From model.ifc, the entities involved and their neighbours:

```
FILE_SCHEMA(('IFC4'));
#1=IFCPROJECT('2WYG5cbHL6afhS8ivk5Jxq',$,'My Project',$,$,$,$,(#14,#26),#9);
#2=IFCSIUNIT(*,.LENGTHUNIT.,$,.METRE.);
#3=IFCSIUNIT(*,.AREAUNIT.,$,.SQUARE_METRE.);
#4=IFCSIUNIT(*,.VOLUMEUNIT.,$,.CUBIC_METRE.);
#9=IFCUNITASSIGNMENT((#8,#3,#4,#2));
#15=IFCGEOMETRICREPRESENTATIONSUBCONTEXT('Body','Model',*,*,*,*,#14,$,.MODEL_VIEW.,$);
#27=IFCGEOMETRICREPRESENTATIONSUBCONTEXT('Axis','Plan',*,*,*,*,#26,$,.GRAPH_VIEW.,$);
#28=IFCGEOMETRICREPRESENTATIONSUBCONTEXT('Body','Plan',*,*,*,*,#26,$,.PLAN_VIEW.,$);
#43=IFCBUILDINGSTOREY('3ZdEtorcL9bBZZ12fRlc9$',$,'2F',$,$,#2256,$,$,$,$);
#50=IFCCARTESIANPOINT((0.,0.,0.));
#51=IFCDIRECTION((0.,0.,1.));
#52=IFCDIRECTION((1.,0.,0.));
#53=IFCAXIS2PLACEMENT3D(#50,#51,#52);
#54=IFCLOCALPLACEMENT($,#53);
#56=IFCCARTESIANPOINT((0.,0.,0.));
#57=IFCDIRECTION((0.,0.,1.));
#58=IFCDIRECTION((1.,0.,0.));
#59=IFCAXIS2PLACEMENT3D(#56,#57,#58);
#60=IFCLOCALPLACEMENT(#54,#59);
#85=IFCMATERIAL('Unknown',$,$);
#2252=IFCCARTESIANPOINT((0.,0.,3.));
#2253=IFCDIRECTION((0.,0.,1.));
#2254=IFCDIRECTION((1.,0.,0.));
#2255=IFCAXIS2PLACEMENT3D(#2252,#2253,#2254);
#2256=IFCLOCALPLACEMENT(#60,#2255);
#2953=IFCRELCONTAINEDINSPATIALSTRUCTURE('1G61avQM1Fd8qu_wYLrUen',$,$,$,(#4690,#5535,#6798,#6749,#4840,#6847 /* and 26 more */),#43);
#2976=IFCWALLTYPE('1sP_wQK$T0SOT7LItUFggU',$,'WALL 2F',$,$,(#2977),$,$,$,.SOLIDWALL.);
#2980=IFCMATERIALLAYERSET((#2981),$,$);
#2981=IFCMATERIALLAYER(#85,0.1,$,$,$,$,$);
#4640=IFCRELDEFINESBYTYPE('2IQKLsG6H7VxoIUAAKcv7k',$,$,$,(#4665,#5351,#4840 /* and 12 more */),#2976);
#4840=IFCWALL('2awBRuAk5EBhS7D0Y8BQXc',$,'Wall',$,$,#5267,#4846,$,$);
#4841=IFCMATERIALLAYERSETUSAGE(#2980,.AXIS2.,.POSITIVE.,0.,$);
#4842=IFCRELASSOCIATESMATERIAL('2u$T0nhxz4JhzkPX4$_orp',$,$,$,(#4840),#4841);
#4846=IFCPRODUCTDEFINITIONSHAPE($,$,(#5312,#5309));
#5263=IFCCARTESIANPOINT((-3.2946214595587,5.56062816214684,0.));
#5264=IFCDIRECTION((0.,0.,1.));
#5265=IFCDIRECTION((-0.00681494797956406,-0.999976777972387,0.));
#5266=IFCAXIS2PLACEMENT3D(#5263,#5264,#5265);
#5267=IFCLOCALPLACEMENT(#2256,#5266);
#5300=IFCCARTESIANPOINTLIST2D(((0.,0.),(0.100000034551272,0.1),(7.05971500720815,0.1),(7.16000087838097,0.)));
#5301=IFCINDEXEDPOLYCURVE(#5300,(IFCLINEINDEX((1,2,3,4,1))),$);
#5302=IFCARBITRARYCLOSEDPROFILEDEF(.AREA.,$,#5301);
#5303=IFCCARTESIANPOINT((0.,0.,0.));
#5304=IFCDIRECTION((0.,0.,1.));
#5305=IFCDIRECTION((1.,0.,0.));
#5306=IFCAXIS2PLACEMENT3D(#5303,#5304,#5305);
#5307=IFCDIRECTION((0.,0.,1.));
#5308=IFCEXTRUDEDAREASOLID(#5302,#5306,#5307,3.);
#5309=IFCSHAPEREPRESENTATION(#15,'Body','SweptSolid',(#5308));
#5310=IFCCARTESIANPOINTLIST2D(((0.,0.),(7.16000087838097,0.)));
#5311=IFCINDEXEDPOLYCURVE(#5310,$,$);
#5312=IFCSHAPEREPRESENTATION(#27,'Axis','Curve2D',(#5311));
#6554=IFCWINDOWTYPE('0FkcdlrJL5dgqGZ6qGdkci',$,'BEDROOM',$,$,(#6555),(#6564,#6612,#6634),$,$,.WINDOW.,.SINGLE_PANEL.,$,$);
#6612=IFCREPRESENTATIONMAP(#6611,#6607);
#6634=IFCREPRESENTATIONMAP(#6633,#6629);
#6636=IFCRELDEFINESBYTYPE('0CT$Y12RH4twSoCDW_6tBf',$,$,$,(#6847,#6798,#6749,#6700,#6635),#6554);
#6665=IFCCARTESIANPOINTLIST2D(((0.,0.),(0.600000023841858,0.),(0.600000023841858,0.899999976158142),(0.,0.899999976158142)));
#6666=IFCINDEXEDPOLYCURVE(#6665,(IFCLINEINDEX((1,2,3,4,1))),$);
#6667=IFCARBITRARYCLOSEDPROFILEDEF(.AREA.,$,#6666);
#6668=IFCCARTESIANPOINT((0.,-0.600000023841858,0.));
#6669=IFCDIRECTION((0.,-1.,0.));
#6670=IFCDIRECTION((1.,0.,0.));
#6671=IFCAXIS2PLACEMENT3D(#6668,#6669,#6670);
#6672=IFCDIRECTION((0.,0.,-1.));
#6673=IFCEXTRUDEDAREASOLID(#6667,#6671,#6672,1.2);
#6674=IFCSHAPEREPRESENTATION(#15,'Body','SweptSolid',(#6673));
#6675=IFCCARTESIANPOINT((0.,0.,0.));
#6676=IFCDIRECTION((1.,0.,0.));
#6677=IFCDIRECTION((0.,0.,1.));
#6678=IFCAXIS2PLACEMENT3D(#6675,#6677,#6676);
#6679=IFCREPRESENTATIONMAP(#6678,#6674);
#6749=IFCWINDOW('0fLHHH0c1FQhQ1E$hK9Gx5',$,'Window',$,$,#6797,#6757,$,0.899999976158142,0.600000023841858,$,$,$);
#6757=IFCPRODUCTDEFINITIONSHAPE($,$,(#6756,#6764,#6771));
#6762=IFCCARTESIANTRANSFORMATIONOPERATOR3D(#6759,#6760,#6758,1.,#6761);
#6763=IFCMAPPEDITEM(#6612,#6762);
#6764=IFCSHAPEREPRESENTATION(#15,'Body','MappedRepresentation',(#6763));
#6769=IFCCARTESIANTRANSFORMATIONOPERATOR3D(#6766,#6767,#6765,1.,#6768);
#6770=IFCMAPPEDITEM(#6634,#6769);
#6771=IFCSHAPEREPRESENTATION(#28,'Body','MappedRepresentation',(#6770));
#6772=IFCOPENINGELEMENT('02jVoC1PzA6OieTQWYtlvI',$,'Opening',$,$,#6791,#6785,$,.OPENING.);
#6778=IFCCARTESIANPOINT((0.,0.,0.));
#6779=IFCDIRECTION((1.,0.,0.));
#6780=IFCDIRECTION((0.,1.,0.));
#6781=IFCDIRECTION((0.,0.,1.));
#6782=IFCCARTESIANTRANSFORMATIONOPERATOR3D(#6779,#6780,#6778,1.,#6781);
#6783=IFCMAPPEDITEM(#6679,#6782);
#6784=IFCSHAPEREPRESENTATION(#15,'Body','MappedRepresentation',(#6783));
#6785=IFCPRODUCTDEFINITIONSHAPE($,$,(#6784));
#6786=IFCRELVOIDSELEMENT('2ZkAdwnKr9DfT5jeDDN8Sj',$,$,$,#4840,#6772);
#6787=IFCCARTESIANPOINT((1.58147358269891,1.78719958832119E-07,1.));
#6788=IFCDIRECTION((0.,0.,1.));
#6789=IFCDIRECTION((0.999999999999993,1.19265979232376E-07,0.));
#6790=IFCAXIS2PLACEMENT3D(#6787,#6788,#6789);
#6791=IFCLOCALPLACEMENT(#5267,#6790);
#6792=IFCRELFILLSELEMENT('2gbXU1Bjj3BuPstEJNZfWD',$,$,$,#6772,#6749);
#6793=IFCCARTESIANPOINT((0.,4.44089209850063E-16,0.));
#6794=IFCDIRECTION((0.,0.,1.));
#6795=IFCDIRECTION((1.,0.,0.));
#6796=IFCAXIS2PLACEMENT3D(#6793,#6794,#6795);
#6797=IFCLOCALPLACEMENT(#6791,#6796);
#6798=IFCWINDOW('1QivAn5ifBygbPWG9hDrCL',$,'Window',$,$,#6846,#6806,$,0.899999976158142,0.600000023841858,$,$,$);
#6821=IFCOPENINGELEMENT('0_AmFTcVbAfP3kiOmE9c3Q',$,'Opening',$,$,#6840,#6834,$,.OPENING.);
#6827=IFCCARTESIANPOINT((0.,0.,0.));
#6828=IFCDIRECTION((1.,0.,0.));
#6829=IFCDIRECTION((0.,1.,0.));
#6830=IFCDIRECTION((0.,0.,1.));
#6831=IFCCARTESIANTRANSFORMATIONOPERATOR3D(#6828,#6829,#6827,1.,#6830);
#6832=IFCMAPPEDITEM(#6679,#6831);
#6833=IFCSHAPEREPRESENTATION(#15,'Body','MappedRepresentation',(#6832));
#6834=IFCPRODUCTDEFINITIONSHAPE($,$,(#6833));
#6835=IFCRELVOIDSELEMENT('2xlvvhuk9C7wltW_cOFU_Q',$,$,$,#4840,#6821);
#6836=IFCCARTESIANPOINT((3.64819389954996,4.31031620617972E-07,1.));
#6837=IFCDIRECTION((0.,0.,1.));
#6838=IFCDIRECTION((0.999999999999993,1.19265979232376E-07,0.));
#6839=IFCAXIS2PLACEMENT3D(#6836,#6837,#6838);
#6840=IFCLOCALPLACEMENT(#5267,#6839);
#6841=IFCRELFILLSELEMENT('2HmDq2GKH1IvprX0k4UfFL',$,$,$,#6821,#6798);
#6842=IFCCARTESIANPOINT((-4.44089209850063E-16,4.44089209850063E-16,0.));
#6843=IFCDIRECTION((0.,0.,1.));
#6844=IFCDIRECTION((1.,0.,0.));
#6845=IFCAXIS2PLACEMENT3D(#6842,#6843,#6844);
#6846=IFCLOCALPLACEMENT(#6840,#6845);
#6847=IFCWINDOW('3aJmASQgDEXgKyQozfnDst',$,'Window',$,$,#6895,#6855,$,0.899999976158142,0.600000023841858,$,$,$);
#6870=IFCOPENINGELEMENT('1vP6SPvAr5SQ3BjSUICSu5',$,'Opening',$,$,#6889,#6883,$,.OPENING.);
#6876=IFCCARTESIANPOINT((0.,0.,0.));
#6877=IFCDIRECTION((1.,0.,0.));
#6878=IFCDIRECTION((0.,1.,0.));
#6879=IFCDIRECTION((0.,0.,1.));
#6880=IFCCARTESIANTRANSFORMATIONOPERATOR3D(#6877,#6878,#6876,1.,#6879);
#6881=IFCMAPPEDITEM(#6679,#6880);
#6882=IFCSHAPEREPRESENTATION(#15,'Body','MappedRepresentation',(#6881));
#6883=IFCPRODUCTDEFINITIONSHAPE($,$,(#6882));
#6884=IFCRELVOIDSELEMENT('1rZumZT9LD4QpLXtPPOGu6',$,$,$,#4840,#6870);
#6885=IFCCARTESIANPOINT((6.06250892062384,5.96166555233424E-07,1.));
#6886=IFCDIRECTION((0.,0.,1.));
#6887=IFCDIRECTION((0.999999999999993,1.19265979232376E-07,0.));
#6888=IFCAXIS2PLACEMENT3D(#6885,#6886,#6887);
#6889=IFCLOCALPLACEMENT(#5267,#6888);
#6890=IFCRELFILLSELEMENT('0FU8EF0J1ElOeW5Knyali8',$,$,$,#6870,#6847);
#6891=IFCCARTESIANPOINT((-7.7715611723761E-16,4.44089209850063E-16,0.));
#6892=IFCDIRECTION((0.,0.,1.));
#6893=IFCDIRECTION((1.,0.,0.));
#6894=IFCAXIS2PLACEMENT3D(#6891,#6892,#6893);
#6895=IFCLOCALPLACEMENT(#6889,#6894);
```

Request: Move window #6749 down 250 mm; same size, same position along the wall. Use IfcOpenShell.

```python
import numpy as np
import ifcopenshell
import ifcopenshell.api.geometry
import ifcopenshell.util.placement
import ifcopenshell.util.unit

model = ifcopenshell.open("model.ifc")
unit_scale = ifcopenshell.util.unit.calculate_unit_scale(model)

window = model.by_guid("0fLHHH0c1FQhQ1E$hK9Gx5")
opening = window.FillsVoids[0].RelatingOpeningElement
dz = -0.25 / unit_scale

shift = np.array([0.0, 0.0, dz])
# The window is placed relative to its opening, so it follows when the opening moves.
matrix = ifcopenshell.util.placement.get_local_placement(opening.ObjectPlacement)
matrix[:3, 3] += shift
ifcopenshell.api.geometry.edit_object_placement(
    model, product=opening, matrix=matrix, is_si=False, should_transform_children=True
)

print(f"moved by {dz * unit_scale:+.3f} m")

model.write("model_v2.ifc")
```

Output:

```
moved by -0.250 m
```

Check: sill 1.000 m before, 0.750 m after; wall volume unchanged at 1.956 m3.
